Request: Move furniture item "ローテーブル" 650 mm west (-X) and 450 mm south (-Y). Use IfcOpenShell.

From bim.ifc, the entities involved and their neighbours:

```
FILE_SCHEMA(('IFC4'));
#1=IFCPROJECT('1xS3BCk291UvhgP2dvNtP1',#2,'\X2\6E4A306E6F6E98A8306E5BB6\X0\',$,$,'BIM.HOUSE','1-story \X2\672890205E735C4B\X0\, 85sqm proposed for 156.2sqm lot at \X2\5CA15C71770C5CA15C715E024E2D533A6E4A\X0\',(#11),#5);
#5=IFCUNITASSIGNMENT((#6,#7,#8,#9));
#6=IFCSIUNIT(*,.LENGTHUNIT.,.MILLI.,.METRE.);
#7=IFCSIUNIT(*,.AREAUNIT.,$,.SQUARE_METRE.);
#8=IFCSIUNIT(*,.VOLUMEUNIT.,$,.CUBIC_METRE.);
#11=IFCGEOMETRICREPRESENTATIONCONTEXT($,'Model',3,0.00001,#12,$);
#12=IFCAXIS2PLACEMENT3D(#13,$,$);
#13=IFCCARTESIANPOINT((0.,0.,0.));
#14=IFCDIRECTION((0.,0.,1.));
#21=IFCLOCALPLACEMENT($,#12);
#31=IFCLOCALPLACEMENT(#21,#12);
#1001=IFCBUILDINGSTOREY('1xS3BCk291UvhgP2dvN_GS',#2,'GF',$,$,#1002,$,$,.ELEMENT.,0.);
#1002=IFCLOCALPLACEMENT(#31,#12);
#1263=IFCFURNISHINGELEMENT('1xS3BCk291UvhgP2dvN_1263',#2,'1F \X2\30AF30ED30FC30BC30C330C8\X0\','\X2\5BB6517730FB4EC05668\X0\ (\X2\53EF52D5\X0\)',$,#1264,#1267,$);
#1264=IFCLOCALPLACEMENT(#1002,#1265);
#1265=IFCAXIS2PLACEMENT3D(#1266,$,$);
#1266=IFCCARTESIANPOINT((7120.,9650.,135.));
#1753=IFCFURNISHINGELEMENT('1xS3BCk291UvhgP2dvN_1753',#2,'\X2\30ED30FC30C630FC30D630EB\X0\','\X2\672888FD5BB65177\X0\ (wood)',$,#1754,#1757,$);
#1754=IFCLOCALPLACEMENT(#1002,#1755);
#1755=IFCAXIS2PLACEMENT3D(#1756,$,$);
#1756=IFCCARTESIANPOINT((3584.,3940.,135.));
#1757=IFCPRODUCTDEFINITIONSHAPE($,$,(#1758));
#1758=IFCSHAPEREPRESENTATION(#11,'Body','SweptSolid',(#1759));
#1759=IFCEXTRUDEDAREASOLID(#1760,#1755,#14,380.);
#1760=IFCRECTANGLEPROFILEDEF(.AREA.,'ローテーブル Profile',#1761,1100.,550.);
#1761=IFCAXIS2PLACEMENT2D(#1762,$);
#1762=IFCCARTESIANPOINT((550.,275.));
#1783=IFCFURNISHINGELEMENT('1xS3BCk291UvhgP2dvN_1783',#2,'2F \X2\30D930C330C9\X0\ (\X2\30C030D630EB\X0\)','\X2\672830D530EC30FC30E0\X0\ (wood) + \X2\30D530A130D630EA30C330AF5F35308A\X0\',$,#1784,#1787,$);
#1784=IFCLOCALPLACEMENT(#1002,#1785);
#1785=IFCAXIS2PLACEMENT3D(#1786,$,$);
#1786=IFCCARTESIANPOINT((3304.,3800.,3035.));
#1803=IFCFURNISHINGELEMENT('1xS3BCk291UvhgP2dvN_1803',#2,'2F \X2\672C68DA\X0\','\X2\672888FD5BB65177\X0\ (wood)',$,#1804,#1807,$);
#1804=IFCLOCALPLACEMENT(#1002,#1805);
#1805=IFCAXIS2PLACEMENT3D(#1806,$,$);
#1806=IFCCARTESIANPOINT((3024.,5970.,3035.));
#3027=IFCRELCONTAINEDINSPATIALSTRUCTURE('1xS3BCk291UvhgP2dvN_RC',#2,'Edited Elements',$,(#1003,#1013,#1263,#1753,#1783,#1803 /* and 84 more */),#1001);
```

```python
import ifcopenshell
import ifcopenshell.api.geometry
import ifcopenshell.util.placement
import ifcopenshell.util.unit

model = ifcopenshell.open("bim.ifc")
unit_scale = ifcopenshell.util.unit.calculate_unit_scale(model)

item = model.by_guid("1xS3BCk291UvhgP2dvN_1753")
matrix = ifcopenshell.util.placement.get_local_placement(item.ObjectPlacement)
matrix[0, 3] -= 0.65 / unit_scale
matrix[1, 3] -= 0.45 / unit_scale
ifcopenshell.api.geometry.edit_object_placement(model, product=item, matrix=matrix, is_si=False)

print(ifcopenshell.util.placement.get_local_placement(item.ObjectPlacement).round(3) + 0.0)

model.write("bim_v2.ifc")
```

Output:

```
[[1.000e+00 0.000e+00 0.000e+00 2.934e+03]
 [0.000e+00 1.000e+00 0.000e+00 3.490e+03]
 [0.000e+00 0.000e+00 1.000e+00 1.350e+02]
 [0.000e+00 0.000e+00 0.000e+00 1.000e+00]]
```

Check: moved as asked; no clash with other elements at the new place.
